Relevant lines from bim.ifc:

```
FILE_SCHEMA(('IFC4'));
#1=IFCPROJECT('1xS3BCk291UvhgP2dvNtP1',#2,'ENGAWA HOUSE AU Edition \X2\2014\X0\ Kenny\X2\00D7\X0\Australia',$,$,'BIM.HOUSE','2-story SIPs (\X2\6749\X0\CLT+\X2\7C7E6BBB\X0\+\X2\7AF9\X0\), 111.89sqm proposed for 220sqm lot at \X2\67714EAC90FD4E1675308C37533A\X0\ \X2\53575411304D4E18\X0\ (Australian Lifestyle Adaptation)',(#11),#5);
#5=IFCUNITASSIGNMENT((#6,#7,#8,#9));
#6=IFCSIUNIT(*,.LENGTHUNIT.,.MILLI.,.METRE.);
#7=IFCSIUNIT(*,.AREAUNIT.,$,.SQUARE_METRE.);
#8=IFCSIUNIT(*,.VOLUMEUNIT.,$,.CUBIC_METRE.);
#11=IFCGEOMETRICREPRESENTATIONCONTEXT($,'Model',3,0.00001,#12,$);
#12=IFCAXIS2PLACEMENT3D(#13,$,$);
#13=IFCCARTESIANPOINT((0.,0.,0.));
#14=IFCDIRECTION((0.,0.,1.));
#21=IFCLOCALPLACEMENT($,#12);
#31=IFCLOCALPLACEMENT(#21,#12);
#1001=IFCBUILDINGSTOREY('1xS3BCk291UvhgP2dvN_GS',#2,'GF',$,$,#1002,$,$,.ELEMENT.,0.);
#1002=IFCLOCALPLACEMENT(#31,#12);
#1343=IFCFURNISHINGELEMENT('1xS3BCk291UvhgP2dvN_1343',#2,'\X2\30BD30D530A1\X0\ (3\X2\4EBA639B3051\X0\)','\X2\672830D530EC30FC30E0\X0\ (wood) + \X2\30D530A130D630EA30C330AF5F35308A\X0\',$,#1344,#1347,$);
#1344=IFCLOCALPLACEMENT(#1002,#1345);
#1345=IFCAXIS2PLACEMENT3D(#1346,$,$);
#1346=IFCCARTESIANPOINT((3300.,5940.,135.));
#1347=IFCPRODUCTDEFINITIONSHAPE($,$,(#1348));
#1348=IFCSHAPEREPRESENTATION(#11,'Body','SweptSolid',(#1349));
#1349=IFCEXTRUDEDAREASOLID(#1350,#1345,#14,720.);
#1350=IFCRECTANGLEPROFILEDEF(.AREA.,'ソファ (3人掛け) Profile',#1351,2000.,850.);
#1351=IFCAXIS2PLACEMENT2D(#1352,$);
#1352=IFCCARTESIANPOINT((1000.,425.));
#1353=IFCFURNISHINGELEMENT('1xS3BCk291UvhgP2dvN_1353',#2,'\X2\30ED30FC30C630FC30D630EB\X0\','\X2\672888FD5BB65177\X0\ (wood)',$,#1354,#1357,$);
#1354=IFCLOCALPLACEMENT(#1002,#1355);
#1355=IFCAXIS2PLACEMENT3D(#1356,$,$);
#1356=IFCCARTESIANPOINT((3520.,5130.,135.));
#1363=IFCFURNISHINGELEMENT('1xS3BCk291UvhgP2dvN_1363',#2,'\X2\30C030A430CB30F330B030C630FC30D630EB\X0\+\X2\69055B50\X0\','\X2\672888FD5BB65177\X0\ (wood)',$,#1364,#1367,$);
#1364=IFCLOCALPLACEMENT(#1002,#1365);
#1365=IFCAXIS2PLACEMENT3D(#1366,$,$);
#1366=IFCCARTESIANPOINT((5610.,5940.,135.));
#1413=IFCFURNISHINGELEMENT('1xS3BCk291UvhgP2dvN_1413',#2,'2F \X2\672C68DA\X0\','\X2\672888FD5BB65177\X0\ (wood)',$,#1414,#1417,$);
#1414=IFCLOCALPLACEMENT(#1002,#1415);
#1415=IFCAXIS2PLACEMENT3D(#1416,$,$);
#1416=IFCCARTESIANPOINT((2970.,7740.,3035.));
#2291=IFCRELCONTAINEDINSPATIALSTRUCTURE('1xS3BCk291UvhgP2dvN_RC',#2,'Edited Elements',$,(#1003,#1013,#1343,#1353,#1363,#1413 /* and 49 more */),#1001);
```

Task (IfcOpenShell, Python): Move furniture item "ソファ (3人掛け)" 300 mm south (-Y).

```python
import ifcopenshell
import ifcopenshell.api.geometry
import ifcopenshell.util.placement
import ifcopenshell.util.unit

model = ifcopenshell.open("bim.ifc")
unit_scale = ifcopenshell.util.unit.calculate_unit_scale(model)

item = model.by_id(1343)
matrix = ifcopenshell.util.placement.get_local_placement(item.ObjectPlacement)
matrix[1, 3] -= 0.3 / unit_scale
ifcopenshell.api.geometry.edit_object_placement(model, product=item, matrix=matrix, is_si=False)

print(ifcopenshell.util.placement.get_local_placement(item.ObjectPlacement).round(3) + 0.0)

model.write("bim_updated.ifc")
```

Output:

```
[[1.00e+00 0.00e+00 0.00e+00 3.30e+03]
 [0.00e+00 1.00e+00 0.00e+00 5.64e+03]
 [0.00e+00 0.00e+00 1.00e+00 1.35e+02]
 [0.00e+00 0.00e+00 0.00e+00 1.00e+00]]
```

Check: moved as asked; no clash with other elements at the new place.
